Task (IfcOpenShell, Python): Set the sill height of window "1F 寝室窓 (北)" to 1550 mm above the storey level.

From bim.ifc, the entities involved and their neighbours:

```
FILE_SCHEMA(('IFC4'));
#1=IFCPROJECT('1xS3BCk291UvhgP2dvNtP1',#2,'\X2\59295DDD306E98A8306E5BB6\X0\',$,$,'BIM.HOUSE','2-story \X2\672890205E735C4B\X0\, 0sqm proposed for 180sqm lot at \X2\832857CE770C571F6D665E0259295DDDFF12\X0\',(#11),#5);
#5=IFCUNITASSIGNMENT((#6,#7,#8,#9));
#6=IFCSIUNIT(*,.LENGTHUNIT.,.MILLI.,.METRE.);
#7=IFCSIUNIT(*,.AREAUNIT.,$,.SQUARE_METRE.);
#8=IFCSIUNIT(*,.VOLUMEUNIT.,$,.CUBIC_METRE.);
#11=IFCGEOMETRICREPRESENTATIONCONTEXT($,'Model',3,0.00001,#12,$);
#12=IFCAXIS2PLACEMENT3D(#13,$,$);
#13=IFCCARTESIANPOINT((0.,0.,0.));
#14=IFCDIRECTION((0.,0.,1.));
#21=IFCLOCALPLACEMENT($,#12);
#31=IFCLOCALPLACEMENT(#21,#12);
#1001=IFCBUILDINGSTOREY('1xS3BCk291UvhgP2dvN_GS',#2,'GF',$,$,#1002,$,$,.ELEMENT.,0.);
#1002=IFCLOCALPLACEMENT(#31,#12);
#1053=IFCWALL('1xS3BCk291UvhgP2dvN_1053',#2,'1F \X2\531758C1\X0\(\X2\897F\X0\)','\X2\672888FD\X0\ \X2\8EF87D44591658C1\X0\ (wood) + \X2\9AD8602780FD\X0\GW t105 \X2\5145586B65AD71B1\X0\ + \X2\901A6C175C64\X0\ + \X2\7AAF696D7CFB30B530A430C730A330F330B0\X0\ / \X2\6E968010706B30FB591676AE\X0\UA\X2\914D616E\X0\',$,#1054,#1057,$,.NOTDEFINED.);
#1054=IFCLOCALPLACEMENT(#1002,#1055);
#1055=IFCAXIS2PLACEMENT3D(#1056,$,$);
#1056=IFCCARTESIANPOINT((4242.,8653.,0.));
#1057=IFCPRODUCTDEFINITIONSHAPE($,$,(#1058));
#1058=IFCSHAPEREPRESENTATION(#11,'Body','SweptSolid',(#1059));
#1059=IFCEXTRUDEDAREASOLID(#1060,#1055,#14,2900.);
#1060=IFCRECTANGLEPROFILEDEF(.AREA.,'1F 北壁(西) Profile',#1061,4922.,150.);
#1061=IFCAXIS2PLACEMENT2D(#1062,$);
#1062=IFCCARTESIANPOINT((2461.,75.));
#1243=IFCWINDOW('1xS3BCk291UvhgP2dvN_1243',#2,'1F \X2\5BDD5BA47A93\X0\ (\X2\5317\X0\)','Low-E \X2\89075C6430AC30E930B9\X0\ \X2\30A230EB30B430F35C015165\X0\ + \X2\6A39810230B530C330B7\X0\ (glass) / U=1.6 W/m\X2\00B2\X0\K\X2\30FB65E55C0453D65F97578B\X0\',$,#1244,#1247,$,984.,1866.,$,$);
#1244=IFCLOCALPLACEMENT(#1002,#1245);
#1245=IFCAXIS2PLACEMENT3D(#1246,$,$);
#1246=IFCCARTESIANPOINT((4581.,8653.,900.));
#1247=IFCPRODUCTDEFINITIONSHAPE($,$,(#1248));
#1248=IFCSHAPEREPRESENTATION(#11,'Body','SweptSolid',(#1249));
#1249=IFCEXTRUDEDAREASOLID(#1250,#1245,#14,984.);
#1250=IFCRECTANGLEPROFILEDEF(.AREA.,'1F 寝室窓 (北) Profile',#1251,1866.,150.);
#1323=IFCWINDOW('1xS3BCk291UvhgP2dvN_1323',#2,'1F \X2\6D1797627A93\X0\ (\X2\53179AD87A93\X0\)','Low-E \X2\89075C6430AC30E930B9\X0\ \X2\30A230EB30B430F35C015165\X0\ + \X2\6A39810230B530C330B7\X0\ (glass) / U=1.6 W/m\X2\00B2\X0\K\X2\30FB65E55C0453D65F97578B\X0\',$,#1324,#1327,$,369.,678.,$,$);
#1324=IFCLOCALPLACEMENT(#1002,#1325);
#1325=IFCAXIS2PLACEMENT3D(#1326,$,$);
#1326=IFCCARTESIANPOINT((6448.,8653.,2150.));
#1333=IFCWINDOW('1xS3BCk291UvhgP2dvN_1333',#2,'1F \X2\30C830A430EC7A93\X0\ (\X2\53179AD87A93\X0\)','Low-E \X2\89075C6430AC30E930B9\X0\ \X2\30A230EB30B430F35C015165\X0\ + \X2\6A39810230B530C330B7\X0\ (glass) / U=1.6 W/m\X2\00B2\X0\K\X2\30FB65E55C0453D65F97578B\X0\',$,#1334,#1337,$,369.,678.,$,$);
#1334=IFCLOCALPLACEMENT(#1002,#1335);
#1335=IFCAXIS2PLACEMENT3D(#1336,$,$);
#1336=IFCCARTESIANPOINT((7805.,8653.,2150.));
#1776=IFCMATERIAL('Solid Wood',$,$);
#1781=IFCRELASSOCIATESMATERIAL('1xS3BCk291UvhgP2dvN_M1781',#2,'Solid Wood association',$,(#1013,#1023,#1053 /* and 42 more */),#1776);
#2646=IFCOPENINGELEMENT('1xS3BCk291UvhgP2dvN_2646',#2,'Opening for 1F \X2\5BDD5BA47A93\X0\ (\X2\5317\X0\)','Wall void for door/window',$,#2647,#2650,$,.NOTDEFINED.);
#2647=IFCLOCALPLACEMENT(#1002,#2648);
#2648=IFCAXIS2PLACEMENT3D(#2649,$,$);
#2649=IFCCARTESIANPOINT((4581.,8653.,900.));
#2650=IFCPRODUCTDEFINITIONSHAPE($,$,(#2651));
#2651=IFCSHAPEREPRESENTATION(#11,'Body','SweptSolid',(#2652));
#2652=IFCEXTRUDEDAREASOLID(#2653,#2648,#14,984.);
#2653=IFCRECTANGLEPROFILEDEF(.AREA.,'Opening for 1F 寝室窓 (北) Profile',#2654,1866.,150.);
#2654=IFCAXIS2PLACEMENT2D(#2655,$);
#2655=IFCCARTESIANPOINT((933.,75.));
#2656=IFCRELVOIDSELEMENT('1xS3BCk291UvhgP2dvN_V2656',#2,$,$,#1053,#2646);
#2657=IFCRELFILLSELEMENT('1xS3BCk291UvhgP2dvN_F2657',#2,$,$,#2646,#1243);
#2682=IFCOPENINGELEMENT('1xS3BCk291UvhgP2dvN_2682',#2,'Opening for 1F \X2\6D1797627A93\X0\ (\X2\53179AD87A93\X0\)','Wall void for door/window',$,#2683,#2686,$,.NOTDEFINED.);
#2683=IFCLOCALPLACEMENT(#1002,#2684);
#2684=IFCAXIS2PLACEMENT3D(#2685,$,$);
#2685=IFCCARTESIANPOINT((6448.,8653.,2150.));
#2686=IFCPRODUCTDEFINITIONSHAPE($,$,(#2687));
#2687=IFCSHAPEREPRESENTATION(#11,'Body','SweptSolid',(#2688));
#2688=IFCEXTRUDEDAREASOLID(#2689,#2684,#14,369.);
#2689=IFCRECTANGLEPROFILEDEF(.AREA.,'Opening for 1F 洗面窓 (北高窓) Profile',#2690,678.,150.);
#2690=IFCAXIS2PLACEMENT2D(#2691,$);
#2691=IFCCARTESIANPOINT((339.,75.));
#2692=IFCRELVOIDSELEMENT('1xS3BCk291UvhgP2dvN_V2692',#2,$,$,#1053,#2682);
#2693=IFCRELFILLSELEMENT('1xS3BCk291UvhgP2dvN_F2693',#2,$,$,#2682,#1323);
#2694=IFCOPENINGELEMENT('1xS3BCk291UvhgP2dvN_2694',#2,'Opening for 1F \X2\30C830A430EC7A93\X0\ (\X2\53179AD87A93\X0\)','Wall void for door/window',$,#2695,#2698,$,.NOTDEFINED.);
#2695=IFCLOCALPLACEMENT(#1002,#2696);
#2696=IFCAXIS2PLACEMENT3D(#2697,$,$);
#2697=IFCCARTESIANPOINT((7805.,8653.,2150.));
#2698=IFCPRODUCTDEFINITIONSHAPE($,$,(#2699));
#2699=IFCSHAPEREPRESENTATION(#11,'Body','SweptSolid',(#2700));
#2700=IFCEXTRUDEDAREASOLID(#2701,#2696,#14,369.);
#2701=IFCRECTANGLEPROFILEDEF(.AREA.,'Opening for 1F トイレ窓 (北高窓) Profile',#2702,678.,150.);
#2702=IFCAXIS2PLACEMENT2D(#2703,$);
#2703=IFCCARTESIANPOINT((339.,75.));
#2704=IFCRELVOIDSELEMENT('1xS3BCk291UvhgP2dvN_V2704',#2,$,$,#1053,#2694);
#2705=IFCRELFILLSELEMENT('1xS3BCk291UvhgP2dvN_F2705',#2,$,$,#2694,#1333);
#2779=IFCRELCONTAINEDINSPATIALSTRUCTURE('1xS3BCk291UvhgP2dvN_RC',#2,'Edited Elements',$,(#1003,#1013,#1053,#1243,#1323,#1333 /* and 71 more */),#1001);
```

```python
import numpy as np
import ifcopenshell
import ifcopenshell.api.geometry
import ifcopenshell.geom
import ifcopenshell.util.element
import ifcopenshell.util.placement
import ifcopenshell.util.shape
import ifcopenshell.util.unit

model = ifcopenshell.open("bim.ifc")
unit_scale = ifcopenshell.util.unit.calculate_unit_scale(model)

window = model.by_guid("1xS3BCk291UvhgP2dvN_1243")
opening = window.FillsVoids[0].RelatingOpeningElement
storey = ifcopenshell.util.element.get_container(window, ifc_class="IfcBuildingStorey")
level = ifcopenshell.util.placement.get_local_placement(storey.ObjectPlacement)[2, 3]

# The opening's origin need not be at the sill, so measure its lowest point.
shape = ifcopenshell.geom.create_shape(ifcopenshell.geom.settings(), opening)
bottom = ifcopenshell.util.shape.get_shape_bottom_elevation(shape, shape.geometry) / unit_scale
dz = level + 1550.0 - bottom

shift = np.array([0.0, 0.0, dz])
# The window is not placed relative to its opening, so move both.
for product in (opening, window):
    matrix = ifcopenshell.util.placement.get_local_placement(product.ObjectPlacement)
    matrix[:3, 3] += shift
    ifcopenshell.api.geometry.edit_object_placement(model, product=product, matrix=matrix, is_si=False)

print(f"moved by {dz * unit_scale:+.3f} m")

model.write("bim_updated.ifc")
```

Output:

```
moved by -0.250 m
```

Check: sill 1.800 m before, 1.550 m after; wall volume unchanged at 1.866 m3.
